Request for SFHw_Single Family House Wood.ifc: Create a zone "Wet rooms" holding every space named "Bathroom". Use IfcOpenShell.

First a look at what the model holds.

```python
import ifcopenshell

model = ifcopenshell.open("SFHw_Single Family House Wood.ifc")
print(model.schema)
seen = {}
for space in model.by_type("IfcSpace"):
    seen[space.LongName] = seen.get(space.LongName, 0) + 1
for name, count in sorted(seen.items(), key=str):
    print(count, "x", name)
print("zones:", [z.Name for z in model.by_type("IfcZone")][:20])
```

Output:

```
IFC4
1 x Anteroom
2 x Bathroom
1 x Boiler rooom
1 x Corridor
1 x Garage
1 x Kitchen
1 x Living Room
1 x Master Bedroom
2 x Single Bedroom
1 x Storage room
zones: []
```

```python
import ifcopenshell
import ifcopenshell.api.group
import ifcopenshell.api.root

model = ifcopenshell.open("SFHw_Single Family House Wood.ifc")

names = {"Bathroom"}
spaces = [s for s in model.by_type("IfcSpace") if s.LongName in names]

zone = ifcopenshell.api.root.create_entity(model, ifc_class="IfcZone", name="Wet rooms")
ifcopenshell.api.group.assign_group(model, products=spaces, group=zone)
print(len(spaces), "spaces in", zone.Name)

model.write("SFHw_Single Family House Wood_updated.ifc")
```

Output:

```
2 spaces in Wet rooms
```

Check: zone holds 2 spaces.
